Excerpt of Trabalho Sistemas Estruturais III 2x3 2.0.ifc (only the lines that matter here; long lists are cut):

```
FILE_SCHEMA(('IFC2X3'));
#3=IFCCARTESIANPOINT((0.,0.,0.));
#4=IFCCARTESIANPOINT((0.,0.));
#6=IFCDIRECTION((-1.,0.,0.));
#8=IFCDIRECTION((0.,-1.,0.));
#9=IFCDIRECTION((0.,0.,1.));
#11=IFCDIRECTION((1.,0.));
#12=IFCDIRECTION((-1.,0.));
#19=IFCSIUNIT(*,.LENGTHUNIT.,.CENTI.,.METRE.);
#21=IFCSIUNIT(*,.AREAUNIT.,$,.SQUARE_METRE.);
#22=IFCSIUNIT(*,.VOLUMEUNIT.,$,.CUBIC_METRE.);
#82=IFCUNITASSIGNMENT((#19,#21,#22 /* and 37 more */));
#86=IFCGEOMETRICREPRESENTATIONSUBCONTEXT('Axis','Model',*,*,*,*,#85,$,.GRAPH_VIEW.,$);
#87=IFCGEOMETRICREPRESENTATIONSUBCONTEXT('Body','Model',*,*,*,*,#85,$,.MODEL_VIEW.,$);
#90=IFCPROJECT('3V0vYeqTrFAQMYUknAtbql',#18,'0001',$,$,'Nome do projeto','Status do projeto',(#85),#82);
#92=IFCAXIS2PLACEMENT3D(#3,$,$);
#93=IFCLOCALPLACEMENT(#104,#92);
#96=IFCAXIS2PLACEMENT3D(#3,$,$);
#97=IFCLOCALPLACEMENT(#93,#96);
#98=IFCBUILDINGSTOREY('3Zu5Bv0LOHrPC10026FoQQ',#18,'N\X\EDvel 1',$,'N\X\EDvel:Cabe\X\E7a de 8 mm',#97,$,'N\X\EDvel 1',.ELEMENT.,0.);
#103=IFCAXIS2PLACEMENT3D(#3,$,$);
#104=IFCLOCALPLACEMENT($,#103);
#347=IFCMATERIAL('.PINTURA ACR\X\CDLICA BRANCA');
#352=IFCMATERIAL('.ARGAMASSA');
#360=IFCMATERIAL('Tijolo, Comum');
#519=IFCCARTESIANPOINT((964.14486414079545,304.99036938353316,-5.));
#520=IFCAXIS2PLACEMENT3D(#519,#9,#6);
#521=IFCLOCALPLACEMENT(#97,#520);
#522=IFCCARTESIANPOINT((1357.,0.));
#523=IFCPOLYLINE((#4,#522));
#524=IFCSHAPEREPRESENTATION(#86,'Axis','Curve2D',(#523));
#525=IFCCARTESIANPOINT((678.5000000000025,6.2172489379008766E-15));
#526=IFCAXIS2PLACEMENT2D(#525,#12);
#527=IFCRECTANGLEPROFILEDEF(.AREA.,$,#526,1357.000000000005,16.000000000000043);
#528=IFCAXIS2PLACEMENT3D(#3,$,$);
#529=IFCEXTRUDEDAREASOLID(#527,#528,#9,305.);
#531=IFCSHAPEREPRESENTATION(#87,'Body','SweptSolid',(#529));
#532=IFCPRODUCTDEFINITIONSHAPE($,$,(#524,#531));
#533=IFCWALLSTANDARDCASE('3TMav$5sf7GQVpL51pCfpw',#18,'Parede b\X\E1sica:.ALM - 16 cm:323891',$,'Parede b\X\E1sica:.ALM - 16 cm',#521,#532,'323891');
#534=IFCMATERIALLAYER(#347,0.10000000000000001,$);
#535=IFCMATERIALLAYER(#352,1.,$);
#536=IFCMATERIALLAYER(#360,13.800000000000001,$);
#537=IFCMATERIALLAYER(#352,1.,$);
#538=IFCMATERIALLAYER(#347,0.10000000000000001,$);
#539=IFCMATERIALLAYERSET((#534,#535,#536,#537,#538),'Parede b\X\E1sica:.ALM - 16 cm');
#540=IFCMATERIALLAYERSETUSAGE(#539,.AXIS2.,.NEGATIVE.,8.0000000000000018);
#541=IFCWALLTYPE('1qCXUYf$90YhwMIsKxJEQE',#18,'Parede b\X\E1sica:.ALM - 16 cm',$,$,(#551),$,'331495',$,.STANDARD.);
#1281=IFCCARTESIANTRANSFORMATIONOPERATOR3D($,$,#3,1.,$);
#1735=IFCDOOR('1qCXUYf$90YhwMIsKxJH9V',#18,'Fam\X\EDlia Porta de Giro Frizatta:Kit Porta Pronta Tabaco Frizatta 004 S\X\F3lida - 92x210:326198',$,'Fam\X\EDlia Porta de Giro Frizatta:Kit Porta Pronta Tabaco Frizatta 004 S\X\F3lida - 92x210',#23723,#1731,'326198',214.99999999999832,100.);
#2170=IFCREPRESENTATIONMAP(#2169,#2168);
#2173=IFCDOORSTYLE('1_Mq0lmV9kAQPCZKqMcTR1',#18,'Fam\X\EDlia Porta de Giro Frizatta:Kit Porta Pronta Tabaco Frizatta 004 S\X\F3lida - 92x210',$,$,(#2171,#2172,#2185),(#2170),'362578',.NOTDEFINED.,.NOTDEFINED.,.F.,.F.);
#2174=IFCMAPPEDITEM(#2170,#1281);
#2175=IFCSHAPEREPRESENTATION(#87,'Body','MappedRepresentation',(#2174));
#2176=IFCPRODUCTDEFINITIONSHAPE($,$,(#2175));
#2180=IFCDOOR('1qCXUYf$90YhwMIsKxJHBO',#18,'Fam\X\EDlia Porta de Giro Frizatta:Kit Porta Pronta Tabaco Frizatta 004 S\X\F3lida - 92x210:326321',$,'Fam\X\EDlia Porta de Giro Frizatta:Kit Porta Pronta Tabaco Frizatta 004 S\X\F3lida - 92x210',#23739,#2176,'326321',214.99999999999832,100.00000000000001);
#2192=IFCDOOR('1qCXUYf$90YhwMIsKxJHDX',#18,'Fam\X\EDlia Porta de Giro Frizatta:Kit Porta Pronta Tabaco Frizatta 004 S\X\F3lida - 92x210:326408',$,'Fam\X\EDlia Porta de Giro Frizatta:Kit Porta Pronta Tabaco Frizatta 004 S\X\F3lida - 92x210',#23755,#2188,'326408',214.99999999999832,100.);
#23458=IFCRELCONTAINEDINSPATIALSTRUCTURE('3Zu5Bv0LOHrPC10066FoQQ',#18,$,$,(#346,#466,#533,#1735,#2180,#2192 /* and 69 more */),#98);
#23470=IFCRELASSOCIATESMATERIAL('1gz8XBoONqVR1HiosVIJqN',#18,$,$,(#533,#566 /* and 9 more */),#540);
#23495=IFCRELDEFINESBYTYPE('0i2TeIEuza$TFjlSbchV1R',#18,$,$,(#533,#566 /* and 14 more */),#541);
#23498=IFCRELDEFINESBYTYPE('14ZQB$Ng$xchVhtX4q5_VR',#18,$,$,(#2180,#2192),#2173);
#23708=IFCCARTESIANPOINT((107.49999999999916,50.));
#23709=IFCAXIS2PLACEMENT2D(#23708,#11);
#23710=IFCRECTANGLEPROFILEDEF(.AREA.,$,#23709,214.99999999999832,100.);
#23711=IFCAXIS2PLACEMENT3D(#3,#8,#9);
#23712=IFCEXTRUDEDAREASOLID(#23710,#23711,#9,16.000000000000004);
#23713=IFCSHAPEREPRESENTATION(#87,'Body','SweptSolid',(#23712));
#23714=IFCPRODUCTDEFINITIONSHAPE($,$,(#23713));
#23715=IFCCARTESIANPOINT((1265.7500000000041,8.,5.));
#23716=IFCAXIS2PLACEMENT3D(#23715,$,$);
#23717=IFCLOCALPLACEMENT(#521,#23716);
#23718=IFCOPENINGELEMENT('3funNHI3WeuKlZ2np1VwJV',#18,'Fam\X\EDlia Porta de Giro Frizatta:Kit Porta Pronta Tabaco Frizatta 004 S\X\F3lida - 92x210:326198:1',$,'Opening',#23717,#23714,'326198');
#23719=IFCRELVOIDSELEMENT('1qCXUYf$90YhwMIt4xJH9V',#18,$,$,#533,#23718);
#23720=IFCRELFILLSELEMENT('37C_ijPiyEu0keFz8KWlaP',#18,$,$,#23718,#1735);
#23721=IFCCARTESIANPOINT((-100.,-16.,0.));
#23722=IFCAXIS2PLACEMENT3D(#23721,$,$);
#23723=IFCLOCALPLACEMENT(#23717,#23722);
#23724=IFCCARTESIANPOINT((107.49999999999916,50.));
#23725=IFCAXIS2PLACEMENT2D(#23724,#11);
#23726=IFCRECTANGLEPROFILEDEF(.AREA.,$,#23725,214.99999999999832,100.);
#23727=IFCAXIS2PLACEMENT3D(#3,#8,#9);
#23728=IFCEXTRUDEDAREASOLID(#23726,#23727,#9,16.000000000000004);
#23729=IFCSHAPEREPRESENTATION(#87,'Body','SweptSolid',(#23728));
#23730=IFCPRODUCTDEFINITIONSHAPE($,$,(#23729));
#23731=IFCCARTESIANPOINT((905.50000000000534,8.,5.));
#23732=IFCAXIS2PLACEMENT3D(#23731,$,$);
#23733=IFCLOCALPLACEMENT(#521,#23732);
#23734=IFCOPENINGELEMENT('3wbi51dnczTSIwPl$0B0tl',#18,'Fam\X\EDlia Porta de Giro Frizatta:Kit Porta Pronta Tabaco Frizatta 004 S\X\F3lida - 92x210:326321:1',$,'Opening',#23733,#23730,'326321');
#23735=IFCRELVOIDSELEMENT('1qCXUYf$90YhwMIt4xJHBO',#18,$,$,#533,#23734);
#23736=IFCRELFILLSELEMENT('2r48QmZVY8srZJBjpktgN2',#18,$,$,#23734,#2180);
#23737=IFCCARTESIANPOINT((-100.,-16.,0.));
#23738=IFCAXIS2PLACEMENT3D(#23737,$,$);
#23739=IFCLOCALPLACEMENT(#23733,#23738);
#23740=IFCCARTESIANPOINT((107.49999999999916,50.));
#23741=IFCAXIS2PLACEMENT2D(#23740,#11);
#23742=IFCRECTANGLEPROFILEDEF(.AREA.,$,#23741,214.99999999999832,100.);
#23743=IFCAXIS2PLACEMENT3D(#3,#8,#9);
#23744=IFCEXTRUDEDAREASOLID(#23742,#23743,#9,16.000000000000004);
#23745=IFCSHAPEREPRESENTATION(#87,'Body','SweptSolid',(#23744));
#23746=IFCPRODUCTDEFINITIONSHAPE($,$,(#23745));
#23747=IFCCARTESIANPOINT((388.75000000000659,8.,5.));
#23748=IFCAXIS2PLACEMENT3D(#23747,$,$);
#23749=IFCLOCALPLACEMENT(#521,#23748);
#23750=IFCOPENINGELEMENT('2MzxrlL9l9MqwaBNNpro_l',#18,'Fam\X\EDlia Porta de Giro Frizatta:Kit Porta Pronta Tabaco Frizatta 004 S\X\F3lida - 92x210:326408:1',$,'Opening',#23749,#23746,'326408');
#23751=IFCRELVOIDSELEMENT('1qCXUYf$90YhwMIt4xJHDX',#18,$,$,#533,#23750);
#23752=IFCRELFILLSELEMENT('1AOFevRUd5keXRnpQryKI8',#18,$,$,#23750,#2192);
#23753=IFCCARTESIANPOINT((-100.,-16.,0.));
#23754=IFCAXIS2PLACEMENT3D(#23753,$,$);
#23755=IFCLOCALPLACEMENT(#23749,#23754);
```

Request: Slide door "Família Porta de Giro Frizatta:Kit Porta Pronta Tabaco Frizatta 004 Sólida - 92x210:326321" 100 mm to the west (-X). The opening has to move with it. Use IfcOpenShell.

```python
import ifcopenshell
import ifcopenshell.api.geometry
import ifcopenshell.util.placement
import ifcopenshell.util.unit

model = ifcopenshell.open("Trabalho Sistemas Estruturais III 2x3 2.0.ifc")
unit_scale = ifcopenshell.util.unit.calculate_unit_scale(model)

door = model.by_guid("1qCXUYf$90YhwMIsKxJHBO")
opening = door.FillsVoids[0].RelatingOpeningElement
wall = opening.VoidsElements[0].RelatingBuildingElement

wall_matrix = ifcopenshell.util.placement.get_local_placement(wall.ObjectPlacement)
shift = wall_matrix[:3, 0] * 0.1 / unit_scale
before = ifcopenshell.util.placement.get_local_placement(door.ObjectPlacement)[:3, 3].copy()

# The door is placed relative to its opening, so it follows when the opening moves.
matrix = ifcopenshell.util.placement.get_local_placement(opening.ObjectPlacement)
matrix[:3, 3] += shift
ifcopenshell.api.geometry.edit_object_placement(
    model, product=opening, matrix=matrix, is_si=False, should_transform_children=True
)

after = ifcopenshell.util.placement.get_local_placement(door.ObjectPlacement)[:3, 3]
print("door moved by", (after - before).round(3) + 0.0)

model.write("Trabalho Sistemas Estruturais III 2x3 2.0_updated.ifc")
```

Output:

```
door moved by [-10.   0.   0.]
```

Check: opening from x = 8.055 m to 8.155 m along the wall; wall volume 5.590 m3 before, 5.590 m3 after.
